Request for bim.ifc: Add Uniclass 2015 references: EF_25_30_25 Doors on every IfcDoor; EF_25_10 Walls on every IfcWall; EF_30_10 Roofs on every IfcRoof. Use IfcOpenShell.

First a look at what the model holds.

```python
import ifcopenshell

model = ifcopenshell.open("bim.ifc")
print(model.schema)
print("classifications:", [c.Name for c in model.by_type("IfcClassification")])
for ifc_class in ("IfcDoor", "IfcRoof", "IfcStair", "IfcWall", "IfcWindow"):
    print(ifc_class, len(model.by_type(ifc_class)))
```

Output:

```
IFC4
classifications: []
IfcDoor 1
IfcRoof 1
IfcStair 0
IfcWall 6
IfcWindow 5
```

```python
import ifcopenshell
import ifcopenshell.api.classification

model = ifcopenshell.open("bim.ifc")

system = ifcopenshell.api.classification.add_classification(model, classification="Uniclass 2015")

codes = {
    "IfcDoor": ("EF_25_30_25", "Doors"),
    "IfcWall": ("EF_25_10", "Walls"),
    "IfcRoof": ("EF_30_10", "Roofs"),
}
for ifc_class, (code, name) in codes.items():
    products = model.by_type(ifc_class)
    ifcopenshell.api.classification.add_reference(
        model, products=products, classification=system, identification=code, name=name
    )
    print(code, len(products))

model.write("bim_rev.ifc")
```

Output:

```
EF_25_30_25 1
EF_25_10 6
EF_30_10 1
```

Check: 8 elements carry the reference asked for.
